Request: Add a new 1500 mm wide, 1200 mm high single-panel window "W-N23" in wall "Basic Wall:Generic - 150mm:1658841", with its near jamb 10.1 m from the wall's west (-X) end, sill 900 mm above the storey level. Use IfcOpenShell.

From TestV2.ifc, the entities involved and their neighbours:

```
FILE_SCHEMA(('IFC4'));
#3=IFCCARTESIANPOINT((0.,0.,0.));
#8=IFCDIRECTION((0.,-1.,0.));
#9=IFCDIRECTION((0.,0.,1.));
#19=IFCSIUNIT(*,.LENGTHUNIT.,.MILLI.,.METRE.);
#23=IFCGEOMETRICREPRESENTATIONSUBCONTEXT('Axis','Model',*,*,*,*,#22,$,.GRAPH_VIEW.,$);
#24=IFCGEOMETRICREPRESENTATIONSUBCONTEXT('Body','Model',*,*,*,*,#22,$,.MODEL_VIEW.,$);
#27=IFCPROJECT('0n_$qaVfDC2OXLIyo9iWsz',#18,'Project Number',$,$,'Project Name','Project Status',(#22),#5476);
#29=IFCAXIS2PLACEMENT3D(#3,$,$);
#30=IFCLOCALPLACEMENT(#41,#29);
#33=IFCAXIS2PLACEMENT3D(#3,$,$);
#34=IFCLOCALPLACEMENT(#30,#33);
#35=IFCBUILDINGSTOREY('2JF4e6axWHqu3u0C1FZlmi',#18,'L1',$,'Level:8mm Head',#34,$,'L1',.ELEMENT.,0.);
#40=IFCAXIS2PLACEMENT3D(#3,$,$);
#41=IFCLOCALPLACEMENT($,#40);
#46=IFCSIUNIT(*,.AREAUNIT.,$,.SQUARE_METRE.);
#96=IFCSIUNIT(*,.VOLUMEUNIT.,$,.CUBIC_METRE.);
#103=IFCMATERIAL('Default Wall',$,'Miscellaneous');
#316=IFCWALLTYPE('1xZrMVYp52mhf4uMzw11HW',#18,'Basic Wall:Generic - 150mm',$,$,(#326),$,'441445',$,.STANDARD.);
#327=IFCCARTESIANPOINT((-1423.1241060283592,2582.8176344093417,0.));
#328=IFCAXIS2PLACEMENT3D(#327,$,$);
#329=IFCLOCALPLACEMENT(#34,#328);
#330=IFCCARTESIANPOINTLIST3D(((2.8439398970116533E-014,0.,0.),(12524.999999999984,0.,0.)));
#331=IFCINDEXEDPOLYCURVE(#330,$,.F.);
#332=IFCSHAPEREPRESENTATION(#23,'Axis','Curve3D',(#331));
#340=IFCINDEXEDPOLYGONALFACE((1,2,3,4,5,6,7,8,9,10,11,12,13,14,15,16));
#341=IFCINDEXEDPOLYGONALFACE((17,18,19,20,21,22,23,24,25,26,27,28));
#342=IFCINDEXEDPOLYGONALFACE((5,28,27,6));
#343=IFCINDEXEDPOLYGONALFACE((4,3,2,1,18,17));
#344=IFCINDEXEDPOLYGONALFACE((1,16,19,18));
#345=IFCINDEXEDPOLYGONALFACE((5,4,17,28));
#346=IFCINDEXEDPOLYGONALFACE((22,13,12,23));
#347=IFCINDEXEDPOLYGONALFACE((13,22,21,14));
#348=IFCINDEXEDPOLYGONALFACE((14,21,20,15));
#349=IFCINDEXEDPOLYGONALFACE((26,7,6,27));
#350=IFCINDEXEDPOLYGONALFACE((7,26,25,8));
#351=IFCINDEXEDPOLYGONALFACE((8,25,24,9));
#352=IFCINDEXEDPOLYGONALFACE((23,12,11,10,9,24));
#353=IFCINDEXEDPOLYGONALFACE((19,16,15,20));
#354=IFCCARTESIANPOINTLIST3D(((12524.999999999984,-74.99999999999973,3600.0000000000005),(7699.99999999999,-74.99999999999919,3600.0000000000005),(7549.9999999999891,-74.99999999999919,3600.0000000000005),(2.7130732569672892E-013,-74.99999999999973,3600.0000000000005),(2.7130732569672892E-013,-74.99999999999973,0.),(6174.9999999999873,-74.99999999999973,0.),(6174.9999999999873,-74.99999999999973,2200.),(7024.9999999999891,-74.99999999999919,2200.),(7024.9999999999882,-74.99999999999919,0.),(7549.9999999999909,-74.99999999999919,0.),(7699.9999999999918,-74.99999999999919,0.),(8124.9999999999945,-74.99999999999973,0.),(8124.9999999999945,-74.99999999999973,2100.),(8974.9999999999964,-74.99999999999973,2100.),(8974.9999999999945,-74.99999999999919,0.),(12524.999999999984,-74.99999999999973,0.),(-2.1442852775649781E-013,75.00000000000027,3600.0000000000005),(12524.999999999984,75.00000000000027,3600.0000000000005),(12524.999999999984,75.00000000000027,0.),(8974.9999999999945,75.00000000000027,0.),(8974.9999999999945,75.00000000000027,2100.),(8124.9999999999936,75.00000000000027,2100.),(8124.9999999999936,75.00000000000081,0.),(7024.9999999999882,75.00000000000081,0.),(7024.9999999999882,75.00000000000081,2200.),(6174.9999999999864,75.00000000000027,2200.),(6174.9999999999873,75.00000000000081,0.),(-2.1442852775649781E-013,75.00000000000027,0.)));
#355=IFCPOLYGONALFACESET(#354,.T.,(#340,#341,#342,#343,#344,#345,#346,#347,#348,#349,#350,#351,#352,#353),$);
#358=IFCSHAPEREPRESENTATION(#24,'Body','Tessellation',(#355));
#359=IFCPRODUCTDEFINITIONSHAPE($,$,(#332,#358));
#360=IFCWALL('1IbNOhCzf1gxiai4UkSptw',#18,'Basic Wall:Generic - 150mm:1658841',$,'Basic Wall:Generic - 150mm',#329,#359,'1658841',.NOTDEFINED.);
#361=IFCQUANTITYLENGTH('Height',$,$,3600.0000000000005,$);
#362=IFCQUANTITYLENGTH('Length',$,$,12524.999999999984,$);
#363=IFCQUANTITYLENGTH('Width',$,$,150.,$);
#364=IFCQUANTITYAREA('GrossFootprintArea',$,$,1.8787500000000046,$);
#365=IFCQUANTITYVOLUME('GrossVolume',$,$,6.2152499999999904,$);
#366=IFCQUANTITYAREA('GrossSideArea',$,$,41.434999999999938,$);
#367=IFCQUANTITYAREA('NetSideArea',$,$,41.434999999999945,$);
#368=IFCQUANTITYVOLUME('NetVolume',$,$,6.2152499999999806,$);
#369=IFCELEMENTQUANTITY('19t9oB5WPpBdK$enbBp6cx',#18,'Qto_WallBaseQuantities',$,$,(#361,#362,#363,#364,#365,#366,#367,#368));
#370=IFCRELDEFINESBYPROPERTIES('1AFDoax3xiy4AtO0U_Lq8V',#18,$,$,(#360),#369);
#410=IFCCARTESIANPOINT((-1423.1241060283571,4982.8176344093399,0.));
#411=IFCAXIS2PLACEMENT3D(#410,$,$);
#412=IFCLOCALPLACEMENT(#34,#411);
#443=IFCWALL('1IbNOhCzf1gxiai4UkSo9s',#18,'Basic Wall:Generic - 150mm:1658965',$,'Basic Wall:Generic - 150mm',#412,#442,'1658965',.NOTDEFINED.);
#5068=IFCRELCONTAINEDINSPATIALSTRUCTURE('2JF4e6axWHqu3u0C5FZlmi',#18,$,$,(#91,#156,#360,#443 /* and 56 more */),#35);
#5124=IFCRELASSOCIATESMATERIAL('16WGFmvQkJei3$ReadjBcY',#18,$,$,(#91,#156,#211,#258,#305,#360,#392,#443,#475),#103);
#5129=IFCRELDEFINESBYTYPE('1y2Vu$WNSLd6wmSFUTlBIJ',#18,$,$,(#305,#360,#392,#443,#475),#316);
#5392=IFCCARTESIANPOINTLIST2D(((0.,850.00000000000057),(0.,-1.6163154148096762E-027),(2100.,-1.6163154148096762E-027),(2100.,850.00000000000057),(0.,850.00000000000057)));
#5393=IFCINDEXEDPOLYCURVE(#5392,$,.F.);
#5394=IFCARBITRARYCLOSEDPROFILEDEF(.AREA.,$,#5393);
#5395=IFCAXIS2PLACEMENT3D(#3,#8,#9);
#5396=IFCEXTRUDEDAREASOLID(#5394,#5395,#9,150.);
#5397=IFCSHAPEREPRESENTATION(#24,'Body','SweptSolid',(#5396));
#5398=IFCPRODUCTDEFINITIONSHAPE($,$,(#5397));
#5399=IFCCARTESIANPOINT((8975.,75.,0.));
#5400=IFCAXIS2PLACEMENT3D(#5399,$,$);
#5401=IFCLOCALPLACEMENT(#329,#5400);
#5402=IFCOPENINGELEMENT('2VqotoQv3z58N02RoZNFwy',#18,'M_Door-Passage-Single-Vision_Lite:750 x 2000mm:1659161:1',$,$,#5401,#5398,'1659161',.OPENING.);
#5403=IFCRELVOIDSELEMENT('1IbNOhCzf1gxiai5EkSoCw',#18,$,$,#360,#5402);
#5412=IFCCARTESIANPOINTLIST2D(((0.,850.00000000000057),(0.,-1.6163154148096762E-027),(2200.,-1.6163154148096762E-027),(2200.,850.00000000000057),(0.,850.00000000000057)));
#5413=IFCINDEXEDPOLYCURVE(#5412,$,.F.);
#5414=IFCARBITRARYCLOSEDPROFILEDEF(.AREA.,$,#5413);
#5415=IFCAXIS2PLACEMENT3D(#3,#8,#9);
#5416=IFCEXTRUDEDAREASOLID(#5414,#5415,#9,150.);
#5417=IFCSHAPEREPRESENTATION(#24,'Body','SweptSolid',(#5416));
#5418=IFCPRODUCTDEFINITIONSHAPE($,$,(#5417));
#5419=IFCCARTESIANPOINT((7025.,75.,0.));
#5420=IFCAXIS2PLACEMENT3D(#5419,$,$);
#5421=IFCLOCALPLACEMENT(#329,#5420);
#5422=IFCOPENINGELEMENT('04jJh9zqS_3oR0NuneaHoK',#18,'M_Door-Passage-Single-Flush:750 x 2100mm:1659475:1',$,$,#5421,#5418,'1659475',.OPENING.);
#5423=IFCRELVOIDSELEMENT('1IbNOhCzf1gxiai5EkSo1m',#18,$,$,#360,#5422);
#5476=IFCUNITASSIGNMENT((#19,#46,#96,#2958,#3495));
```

```python
import numpy as np
import ifcopenshell
import ifcopenshell.api.feature
import ifcopenshell.api.geometry
import ifcopenshell.api.pset
import ifcopenshell.api.root
import ifcopenshell.api.spatial
import ifcopenshell.geom
import ifcopenshell.util.element
import ifcopenshell.util.placement
import ifcopenshell.util.representation
import ifcopenshell.util.shape
import ifcopenshell.util.unit

model = ifcopenshell.open("TestV2.ifc")
unit_scale = ifcopenshell.util.unit.calculate_unit_scale(model)
area_scale = ifcopenshell.util.unit.calculate_unit_scale(model, "AREAUNIT")
volume_scale = ifcopenshell.util.unit.calculate_unit_scale(model, "VOLUMEUNIT")
settings = ifcopenshell.geom.settings()


def volume(element):
    """Net volume in cubic metres, openings subtracted."""
    shape = ifcopenshell.geom.create_shape(settings, element)
    return ifcopenshell.util.shape.get_volume(shape.geometry)


wall = model.by_guid("1IbNOhCzf1gxiai4UkSptw")
storey = ifcopenshell.util.element.get_container(wall, ifc_class="IfcBuildingStorey")
context = ifcopenshell.util.representation.get_context(model, "Model", "Body", "MODEL_VIEW")
before = volume(wall)

width, height, from_end, sill = 1.5, 1.2, 10.1, 0.9  # metres

# The wall runs along its own X axis, and the end named is its -X end.
wall_shape = ifcopenshell.geom.create_shape(settings, wall)
x, y, z = ifcopenshell.util.shape.get_vertices(wall_shape.geometry).T
start = x.min() + from_end
face, thickness = float(y.min()), float(y.max() - y.min())
wall_matrix = ifcopenshell.util.placement.get_local_placement(wall.ObjectPlacement)
level = ifcopenshell.util.placement.get_local_placement(storey.ObjectPlacement)[2, 3]


def in_wall(x, y):
    """Placement at x, y metres in the wall's axes, at sill height."""
    matrix = wall_matrix.copy()
    matrix[:, 3] = wall_matrix @ np.array([x / unit_scale, y / unit_scale, 0.0, 1.0])
    matrix[2, 3] = level + sill / unit_scale
    return matrix


# Opening: a box that overshoots both wall faces by 50 mm.
opening = ifcopenshell.api.root.create_entity(model, ifc_class="IfcOpeningElement", predefined_type="OPENING")
box = ifcopenshell.api.geometry.add_wall_representation(
    model, context=context, length=width, height=height, thickness=thickness + 0.1
)
ifcopenshell.api.geometry.assign_representation(model, product=opening, representation=box)
ifcopenshell.api.geometry.edit_object_placement(model, product=opening, matrix=in_wall(start, face - 0.05), is_si=False)
ifcopenshell.api.feature.add_feature(model, feature=opening, element=wall)

window = ifcopenshell.api.root.create_entity(model, ifc_class="IfcWindow", name="W-N23", predefined_type="WINDOW")
window.OverallWidth, window.OverallHeight = width / unit_scale, height / unit_scale
window.PartitioningType = "SINGLE_PANEL"
body = ifcopenshell.api.geometry.add_window_representation(
    model,
    context=context,
    overall_width=window.OverallWidth,
    overall_height=window.OverallHeight,
    partition_type="SINGLE_PANEL",
)
ifcopenshell.api.geometry.assign_representation(model, product=window, representation=body)
ifcopenshell.api.spatial.assign_container(model, products=[window], relating_structure=storey)
ifcopenshell.api.feature.add_filling(model, opening=opening, element=window)

# Centre the window in the wall's thickness.
ifcopenshell.api.geometry.edit_object_placement(model, product=window, matrix=in_wall(start, face), is_si=False)
window_shape = ifcopenshell.geom.create_shape(settings, window)
depth = ifcopenshell.util.shape.get_vertices(window_shape.geometry)[:, 1]
offset = face + thickness / 2 - (depth.min() + depth.max()) / 2
ifcopenshell.api.geometry.edit_object_placement(model, product=window, matrix=in_wall(start, offset), is_si=False)

after = volume(wall)

# Update the wall's stored quantities.
qto = model.by_id(ifcopenshell.util.element.get_pset(wall, "Qto_WallBaseQuantities", should_inherit=False)["id"])
ifcopenshell.api.pset.edit_qto(model, qto=qto, properties={
    "NetSideArea": after / thickness / area_scale,
    "NetVolume": after / volume_scale,
})

print(f"wall volume {before:.3f} -> {after:.3f} m3")

model.write("TestV2_edited.ifc")
```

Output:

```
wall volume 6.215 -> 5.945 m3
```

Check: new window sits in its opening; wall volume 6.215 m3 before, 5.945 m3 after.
